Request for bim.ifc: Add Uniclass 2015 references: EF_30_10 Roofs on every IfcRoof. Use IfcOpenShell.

First a look at what the model holds.

```python
import ifcopenshell

model = ifcopenshell.open("bim.ifc")
print(model.schema)
print("classifications:", [c.Name for c in model.by_type("IfcClassification")])
for ifc_class in ("IfcDoor", "IfcRoof", "IfcStair", "IfcWall", "IfcWindow"):
    print(ifc_class, len(model.by_type(ifc_class)))
```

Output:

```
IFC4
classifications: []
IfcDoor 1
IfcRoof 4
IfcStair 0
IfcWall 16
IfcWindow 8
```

```python
import ifcopenshell
import ifcopenshell.api.classification

model = ifcopenshell.open("bim.ifc")

system = ifcopenshell.api.classification.add_classification(model, classification="Uniclass 2015")

codes = {
    "IfcRoof": ("EF_30_10", "Roofs"),
}
for ifc_class, (code, name) in codes.items():
    products = model.by_type(ifc_class)
    ifcopenshell.api.classification.add_reference(
        model, products=products, classification=system, identification=code, name=name
    )
    print(code, len(products))

model.write("bim_rev.ifc")
```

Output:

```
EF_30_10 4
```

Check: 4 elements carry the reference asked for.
